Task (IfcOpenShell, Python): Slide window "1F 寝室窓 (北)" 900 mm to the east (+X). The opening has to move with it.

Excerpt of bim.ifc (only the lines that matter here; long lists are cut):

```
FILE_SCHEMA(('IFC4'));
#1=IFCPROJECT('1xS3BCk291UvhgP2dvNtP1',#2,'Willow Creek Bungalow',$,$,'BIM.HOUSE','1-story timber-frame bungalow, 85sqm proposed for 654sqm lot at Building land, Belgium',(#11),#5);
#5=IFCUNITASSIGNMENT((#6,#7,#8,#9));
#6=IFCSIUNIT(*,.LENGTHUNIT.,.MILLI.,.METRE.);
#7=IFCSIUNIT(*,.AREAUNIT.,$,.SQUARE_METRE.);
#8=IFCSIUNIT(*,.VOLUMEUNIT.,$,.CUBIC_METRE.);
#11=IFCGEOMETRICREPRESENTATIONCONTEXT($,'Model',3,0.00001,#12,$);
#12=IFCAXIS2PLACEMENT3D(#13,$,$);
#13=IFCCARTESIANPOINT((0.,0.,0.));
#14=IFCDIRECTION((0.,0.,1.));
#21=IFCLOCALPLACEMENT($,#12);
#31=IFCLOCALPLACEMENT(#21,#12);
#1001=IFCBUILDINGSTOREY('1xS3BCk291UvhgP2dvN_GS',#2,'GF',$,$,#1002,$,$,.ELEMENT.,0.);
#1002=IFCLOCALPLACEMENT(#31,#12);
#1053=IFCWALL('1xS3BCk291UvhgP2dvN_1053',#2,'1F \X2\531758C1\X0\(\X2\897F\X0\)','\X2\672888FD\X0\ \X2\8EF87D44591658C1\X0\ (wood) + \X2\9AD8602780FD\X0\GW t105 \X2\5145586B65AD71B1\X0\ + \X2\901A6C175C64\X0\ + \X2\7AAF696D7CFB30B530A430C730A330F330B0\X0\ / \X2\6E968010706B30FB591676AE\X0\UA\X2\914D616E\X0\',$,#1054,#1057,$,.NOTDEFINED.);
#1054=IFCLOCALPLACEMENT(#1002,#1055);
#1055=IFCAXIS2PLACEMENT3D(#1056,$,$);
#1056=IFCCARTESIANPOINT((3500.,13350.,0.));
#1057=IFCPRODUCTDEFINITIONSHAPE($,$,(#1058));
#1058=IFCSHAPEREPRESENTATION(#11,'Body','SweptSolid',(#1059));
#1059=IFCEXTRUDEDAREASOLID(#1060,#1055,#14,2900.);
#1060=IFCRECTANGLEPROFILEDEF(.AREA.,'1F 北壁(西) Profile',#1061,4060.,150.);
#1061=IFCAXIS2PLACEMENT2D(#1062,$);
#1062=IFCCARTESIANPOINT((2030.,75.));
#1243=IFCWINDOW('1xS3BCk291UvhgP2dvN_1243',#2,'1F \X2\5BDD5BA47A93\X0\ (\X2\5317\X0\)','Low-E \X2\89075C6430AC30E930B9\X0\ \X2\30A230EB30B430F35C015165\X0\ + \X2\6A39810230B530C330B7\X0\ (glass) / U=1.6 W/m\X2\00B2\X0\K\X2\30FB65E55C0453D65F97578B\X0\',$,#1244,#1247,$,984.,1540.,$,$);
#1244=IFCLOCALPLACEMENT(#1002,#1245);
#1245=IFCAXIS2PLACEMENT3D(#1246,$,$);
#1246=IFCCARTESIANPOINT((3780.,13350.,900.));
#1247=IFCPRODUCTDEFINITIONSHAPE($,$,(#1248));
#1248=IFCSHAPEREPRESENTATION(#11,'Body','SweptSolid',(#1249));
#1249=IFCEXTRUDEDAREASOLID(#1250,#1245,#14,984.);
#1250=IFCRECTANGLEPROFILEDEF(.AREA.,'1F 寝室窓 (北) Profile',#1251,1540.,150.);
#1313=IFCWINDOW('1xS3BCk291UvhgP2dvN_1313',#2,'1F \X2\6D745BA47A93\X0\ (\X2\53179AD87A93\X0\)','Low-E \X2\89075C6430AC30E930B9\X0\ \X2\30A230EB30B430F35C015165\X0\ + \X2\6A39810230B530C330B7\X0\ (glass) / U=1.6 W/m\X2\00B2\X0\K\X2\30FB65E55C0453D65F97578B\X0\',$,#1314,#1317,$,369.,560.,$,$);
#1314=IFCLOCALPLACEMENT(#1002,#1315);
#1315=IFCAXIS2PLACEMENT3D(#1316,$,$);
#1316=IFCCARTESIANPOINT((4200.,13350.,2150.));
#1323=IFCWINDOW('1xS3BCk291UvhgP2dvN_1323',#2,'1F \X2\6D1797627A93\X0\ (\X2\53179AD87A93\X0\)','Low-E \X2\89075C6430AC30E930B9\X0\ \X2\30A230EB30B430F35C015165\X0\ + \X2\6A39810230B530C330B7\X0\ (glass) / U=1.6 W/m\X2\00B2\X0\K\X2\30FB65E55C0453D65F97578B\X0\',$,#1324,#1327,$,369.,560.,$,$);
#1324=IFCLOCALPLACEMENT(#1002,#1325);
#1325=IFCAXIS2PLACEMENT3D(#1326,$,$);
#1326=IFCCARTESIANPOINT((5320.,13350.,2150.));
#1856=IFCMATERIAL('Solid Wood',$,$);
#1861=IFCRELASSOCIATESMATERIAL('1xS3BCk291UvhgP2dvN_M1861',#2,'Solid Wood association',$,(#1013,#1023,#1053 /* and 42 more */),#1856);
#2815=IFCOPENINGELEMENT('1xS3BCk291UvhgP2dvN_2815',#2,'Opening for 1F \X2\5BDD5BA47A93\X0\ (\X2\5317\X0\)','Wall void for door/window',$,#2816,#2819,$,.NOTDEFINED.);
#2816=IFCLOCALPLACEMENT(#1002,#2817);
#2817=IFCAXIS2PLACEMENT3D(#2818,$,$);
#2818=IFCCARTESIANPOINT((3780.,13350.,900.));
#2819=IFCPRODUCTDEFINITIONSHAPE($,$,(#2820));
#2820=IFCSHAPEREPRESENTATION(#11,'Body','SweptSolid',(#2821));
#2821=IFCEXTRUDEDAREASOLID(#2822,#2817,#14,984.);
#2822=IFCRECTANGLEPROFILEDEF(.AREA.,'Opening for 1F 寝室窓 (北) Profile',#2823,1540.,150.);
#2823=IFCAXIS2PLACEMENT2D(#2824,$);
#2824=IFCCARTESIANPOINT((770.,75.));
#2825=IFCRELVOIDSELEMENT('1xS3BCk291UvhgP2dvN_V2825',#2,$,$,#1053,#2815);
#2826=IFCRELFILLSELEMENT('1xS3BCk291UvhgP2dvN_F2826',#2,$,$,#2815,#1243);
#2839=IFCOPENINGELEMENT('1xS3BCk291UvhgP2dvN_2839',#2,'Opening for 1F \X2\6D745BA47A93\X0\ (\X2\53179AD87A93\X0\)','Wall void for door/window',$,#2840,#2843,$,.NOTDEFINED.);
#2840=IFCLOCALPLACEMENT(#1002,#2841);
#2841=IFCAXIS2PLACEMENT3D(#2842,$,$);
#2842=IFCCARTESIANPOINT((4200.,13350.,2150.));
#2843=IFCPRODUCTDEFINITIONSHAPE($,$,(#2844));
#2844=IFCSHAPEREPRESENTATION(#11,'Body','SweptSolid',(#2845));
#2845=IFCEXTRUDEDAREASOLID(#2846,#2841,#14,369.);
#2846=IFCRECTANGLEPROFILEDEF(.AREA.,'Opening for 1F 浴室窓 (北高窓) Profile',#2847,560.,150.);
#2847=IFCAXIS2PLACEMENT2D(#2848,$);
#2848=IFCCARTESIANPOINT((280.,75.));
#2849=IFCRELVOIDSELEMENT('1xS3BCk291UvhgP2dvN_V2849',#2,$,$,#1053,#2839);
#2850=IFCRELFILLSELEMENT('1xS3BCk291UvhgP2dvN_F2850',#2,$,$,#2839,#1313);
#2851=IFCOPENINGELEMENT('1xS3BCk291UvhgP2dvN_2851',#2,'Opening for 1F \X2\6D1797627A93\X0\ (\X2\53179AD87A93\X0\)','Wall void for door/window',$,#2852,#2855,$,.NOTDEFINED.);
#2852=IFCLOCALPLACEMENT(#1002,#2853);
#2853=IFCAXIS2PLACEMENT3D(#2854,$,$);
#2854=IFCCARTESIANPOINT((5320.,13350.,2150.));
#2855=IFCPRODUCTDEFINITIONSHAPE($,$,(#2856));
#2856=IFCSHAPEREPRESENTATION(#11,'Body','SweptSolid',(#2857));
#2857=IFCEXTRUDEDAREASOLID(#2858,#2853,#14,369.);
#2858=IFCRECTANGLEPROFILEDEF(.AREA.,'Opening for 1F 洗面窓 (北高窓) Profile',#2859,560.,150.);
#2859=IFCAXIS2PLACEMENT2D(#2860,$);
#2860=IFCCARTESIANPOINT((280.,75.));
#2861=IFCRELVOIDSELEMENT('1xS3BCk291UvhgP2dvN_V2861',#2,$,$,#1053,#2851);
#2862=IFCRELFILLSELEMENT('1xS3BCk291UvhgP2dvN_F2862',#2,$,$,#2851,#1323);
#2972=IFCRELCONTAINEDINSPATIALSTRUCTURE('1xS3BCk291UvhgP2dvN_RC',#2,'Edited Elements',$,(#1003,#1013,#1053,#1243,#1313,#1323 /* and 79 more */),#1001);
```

```python
import ifcopenshell
import ifcopenshell.api.geometry
import ifcopenshell.util.placement

model = ifcopenshell.open("bim.ifc")

window = model.by_guid("1xS3BCk291UvhgP2dvN_1243")
opening = window.FillsVoids[0].RelatingOpeningElement
wall = opening.VoidsElements[0].RelatingBuildingElement

wall_matrix = ifcopenshell.util.placement.get_local_placement(wall.ObjectPlacement)
shift = wall_matrix[:3, 0] * 900.0
before = ifcopenshell.util.placement.get_local_placement(window.ObjectPlacement)[:3, 3].copy()

# The window is not placed relative to its opening, so move both.
for product in (opening, window):
    matrix = ifcopenshell.util.placement.get_local_placement(product.ObjectPlacement)
    matrix[:3, 3] += shift
    ifcopenshell.api.geometry.edit_object_placement(model, product=product, matrix=matrix, is_si=False)

after = ifcopenshell.util.placement.get_local_placement(window.ObjectPlacement)[:3, 3]
print("window moved by", (after - before).round(3) + 0.0)

model.write("bim_updated.ifc")
```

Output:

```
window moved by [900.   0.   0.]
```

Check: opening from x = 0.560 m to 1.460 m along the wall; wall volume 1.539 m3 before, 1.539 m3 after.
